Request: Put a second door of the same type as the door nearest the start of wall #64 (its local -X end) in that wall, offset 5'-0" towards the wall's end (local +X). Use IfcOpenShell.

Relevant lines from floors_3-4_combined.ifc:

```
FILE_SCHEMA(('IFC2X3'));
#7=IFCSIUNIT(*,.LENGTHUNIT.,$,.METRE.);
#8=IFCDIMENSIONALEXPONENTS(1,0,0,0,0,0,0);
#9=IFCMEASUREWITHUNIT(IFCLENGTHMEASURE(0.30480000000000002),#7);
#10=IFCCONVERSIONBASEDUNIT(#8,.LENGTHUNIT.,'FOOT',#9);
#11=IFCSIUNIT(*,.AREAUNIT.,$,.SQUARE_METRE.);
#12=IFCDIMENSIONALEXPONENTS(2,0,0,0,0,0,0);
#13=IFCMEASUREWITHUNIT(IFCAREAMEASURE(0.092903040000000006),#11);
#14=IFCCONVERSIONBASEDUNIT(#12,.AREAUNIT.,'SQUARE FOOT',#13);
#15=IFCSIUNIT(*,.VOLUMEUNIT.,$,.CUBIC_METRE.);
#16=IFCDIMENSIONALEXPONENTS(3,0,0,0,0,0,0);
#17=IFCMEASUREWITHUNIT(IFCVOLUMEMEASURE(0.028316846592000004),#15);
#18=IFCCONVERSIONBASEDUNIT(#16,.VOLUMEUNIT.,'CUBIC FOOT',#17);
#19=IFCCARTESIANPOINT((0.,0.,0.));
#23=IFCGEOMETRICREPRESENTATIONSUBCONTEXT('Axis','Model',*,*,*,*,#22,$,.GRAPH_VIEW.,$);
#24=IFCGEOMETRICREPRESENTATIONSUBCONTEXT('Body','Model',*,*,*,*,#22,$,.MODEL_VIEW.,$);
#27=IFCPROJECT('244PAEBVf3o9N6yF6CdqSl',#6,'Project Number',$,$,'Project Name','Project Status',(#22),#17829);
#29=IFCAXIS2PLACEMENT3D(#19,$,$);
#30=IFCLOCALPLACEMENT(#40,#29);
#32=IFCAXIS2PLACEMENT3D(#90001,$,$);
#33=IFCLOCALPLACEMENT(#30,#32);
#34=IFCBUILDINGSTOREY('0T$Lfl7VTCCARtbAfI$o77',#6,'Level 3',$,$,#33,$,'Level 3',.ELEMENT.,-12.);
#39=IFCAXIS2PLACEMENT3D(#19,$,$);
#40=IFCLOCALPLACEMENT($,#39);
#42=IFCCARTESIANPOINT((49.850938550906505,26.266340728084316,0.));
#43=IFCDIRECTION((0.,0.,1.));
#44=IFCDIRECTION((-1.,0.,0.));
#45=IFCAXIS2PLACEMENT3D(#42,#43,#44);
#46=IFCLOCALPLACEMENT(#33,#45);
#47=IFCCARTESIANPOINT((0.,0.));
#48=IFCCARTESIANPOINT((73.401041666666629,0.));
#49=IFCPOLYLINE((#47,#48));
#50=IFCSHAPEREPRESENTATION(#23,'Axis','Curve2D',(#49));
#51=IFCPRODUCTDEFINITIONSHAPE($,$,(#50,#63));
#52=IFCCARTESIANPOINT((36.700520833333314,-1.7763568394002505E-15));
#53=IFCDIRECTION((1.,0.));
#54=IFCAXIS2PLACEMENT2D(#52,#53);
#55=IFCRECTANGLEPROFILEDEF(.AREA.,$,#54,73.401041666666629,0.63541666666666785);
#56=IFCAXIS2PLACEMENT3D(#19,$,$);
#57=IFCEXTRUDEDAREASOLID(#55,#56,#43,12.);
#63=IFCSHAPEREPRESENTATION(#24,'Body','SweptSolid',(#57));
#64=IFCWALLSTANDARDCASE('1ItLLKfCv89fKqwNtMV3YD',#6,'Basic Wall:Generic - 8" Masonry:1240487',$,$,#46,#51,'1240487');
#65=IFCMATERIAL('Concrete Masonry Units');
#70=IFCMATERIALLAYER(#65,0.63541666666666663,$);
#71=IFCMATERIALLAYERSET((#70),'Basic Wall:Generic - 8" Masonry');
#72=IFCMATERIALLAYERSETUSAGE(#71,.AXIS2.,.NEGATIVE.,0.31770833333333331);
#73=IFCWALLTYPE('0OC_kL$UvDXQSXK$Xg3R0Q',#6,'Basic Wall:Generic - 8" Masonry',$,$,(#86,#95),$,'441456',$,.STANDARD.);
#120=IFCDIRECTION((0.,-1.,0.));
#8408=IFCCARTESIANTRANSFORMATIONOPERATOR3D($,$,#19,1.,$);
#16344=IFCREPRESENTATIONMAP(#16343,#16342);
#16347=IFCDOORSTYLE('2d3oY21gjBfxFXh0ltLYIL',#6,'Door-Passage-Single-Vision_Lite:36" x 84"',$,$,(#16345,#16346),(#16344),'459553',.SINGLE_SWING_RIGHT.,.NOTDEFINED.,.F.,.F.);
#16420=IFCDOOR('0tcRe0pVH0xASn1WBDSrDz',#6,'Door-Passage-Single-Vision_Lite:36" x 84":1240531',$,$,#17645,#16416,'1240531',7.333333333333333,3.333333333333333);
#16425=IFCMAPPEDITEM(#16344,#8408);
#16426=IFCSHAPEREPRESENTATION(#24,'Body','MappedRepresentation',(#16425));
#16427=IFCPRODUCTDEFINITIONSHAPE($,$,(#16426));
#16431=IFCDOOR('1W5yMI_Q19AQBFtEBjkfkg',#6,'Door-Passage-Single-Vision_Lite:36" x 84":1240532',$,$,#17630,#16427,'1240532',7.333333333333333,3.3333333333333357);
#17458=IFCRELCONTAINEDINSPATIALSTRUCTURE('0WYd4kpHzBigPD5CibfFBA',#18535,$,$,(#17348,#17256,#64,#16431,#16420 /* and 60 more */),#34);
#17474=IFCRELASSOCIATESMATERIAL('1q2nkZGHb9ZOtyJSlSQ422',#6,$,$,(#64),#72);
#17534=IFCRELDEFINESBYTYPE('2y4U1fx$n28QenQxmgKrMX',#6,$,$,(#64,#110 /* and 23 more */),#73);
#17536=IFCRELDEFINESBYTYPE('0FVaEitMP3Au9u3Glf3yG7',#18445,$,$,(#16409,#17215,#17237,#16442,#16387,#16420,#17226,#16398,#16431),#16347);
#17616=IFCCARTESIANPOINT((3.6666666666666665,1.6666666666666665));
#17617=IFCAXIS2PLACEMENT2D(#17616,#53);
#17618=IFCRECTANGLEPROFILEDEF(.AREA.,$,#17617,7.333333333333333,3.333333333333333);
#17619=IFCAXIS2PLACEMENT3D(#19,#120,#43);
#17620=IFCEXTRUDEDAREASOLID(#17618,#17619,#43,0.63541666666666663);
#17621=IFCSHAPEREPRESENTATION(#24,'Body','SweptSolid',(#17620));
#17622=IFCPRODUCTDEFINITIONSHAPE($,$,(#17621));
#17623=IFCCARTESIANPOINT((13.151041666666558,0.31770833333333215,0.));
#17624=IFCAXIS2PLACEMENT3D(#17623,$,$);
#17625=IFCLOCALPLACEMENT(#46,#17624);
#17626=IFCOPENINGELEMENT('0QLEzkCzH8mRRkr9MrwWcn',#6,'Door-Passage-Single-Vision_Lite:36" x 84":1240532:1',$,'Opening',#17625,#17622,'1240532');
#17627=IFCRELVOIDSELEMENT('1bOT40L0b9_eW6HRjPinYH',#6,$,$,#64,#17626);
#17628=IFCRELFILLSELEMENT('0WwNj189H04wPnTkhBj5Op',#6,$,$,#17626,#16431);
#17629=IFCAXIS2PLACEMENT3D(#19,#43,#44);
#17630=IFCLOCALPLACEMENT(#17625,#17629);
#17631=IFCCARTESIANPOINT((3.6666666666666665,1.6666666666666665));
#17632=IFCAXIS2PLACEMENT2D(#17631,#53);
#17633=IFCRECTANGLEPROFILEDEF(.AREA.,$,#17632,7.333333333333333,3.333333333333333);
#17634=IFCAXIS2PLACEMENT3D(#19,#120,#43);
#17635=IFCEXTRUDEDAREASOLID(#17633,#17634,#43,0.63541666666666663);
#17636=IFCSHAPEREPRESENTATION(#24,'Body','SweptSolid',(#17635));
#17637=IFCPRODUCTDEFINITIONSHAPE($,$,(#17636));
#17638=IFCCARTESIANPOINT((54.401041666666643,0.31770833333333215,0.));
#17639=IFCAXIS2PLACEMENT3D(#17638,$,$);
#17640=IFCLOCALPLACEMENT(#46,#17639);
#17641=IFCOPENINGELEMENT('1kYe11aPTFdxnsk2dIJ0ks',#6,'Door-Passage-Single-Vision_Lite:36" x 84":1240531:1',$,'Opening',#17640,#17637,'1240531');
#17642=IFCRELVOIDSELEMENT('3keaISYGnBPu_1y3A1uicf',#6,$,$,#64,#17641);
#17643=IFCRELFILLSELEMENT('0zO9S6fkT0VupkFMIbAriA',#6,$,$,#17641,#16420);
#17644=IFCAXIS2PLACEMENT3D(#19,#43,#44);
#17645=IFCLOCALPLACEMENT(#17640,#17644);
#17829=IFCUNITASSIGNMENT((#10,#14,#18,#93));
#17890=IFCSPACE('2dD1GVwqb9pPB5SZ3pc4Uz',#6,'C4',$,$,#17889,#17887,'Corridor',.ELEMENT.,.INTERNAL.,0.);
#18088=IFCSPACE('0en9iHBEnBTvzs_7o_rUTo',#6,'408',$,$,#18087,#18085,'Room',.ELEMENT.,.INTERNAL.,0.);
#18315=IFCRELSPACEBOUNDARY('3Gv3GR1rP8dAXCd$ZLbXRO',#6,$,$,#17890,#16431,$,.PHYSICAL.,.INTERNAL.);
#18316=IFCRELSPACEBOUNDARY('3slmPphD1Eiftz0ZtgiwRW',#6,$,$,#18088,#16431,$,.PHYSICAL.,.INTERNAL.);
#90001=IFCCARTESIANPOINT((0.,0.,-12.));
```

```python
import ifcopenshell
import ifcopenshell.api.feature
import ifcopenshell.api.geometry
import ifcopenshell.api.root
import ifcopenshell.geom
import ifcopenshell.util.element
import ifcopenshell.util.placement
import ifcopenshell.util.shape
import ifcopenshell.util.unit

model = ifcopenshell.open("floors_3-4_combined.ifc")
unit_scale = ifcopenshell.util.unit.calculate_unit_scale(model)
settings = ifcopenshell.geom.settings()


def volume(element):
    """Net volume in cubic metres, openings subtracted."""
    shape = ifcopenshell.geom.create_shape(settings, element)
    return ifcopenshell.util.shape.get_volume(shape.geometry)


def reuse_history(source, copy):
    """copy_class also copies each property set's owner history, people and application; keep the originals."""
    for rel in copy.IsDefinedBy:
        if rel.is_a("IfcRelDefinesByProperties") and (history := rel.RelatingPropertyDefinition.OwnerHistory):
            rel.RelatingPropertyDefinition.OwnerHistory = source.OwnerHistory
            ifcopenshell.util.element.remove_deep2(model, history)


door = model.by_guid("1W5yMI_Q19AQBFtEBjkfkg")
opening = door.FillsVoids[0].RelatingOpeningElement
wall = opening.VoidsElements[0].RelatingBuildingElement
before = volume(wall)
shift = ifcopenshell.util.placement.get_local_placement(wall.ObjectPlacement)[:3, 0] * 60 * 0.0254 / unit_scale

# copy_class copies the void relationship, type, container and properties, but no geometry.
new_opening = ifcopenshell.api.root.copy_class(model, product=opening)
new_opening.Representation = ifcopenshell.util.element.copy_deep(
    model, opening.Representation, exclude=["IfcGeometricRepresentationContext", "IfcRepresentationMap"]
)
new_opening.Name = 'Door-Passage-Single-Vision_Lite:36" x 84"'
new_opening.Tag = None
new_door = ifcopenshell.api.root.copy_class(model, product=door)
new_door.Representation = ifcopenshell.util.element.copy_deep(
    model, door.Representation, exclude=["IfcGeometricRepresentationContext", "IfcRepresentationMap"]
)
new_door.Name = 'Door-Passage-Single-Vision_Lite:36" x 84"'
new_door.Tag = None
reuse_history(door, new_door)
fills = ifcopenshell.api.feature.add_filling(model, opening=new_opening, element=new_door)
fills.OwnerHistory = new_door.OwnerHistory  # required in IFC2X3

for old, new in ((opening, new_opening), (door, new_door)):
    matrix = ifcopenshell.util.placement.get_local_placement(old.ObjectPlacement)
    matrix[:3, 3] += shift
    ifcopenshell.api.geometry.edit_object_placement(model, product=new, matrix=matrix, is_si=False)

after = volume(wall)

print(f"wall volume {before:.3f} -> {after:.3f} m3")

model.write("floors_3-4_combined_v2.ifc")
```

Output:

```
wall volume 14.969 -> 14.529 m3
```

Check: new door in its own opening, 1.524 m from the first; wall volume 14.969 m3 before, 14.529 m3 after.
